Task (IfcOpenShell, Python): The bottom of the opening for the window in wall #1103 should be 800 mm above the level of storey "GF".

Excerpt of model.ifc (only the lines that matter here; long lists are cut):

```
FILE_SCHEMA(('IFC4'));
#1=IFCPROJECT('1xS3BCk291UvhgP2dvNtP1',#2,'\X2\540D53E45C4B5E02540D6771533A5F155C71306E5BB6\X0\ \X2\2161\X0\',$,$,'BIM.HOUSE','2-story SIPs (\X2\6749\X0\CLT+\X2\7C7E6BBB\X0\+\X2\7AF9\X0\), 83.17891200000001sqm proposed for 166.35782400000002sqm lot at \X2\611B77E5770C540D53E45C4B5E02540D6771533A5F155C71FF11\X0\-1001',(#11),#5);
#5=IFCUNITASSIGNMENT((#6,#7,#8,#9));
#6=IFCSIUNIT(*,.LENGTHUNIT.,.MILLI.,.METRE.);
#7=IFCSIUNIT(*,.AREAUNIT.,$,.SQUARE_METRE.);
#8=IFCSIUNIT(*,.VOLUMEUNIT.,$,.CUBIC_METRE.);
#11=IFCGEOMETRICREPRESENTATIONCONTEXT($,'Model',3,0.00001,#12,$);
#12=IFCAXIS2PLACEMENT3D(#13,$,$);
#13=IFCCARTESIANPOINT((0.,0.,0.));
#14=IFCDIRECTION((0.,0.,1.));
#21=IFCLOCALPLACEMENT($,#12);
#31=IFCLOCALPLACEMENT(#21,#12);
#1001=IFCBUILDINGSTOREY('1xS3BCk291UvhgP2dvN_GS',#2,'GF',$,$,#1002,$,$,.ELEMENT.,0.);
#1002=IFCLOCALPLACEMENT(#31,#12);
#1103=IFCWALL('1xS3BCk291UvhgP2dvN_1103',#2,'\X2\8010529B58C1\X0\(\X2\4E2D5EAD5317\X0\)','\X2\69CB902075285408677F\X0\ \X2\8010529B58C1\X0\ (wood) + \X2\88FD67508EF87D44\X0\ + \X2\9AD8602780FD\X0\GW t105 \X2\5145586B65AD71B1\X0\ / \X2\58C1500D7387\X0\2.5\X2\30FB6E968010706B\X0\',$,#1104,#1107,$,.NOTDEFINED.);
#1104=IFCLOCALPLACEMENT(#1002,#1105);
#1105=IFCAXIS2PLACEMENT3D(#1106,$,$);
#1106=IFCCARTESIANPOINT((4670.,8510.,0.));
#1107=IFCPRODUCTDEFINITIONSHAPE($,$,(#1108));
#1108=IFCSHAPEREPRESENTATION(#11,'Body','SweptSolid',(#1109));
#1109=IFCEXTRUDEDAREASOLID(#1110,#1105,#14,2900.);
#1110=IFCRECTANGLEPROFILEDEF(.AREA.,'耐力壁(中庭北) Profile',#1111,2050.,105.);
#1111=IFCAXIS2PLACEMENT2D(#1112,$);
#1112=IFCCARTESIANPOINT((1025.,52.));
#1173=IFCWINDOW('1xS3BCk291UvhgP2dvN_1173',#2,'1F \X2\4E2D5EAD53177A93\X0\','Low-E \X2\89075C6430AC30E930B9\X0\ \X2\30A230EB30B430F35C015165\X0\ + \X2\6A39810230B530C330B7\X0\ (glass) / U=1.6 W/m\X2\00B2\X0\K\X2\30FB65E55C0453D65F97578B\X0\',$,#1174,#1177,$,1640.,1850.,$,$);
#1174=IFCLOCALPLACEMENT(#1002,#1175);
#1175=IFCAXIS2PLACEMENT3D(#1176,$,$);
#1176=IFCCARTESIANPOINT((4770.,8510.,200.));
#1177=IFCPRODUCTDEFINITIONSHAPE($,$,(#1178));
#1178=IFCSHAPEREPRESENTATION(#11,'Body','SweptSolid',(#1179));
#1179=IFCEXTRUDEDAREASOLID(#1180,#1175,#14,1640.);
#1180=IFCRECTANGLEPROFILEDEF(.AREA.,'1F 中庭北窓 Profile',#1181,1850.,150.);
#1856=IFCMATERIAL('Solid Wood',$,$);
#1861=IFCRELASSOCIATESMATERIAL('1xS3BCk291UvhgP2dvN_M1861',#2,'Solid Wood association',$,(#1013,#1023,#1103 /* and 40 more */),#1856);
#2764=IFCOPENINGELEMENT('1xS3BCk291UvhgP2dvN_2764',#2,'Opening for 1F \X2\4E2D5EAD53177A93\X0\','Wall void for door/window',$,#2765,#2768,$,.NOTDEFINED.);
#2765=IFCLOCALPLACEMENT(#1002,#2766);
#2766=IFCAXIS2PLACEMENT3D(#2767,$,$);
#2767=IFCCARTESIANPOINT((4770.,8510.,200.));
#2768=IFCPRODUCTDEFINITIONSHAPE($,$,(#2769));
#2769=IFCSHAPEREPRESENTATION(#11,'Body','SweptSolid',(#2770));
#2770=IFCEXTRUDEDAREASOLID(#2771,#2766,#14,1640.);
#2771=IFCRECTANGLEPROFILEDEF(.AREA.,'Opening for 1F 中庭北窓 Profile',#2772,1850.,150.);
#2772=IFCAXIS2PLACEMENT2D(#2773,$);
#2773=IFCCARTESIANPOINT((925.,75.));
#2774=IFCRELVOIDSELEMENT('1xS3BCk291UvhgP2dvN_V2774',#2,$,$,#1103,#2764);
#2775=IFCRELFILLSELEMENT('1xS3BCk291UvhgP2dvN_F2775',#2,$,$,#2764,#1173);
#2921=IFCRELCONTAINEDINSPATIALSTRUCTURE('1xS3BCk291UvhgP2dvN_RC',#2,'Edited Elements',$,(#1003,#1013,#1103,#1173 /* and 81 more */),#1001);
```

```python
import numpy as np
import ifcopenshell
import ifcopenshell.api.geometry
import ifcopenshell.geom
import ifcopenshell.util.element
import ifcopenshell.util.placement
import ifcopenshell.util.shape
import ifcopenshell.util.unit

model = ifcopenshell.open("model.ifc")
unit_scale = ifcopenshell.util.unit.calculate_unit_scale(model)

window = model.by_guid("1xS3BCk291UvhgP2dvN_1173")
opening = window.FillsVoids[0].RelatingOpeningElement
storey = ifcopenshell.util.element.get_container(window, ifc_class="IfcBuildingStorey")
level = ifcopenshell.util.placement.get_local_placement(storey.ObjectPlacement)[2, 3]

# The opening's origin need not be at the sill, so measure its lowest point.
shape = ifcopenshell.geom.create_shape(ifcopenshell.geom.settings(), opening)
bottom = ifcopenshell.util.shape.get_shape_bottom_elevation(shape, shape.geometry) / unit_scale
dz = level + 0.8 / unit_scale - bottom

shift = np.array([0.0, 0.0, dz])
# The window is not placed relative to its opening, so move both.
for product in (opening, window):
    matrix = ifcopenshell.util.placement.get_local_placement(product.ObjectPlacement)
    matrix[:3, 3] += shift
    ifcopenshell.api.geometry.edit_object_placement(model, product=product, matrix=matrix, is_si=False)

print(f"moved by {dz * unit_scale:+.3f} m")

model.write("model-out.ifc")
```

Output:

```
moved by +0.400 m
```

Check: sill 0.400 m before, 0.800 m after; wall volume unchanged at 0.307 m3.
